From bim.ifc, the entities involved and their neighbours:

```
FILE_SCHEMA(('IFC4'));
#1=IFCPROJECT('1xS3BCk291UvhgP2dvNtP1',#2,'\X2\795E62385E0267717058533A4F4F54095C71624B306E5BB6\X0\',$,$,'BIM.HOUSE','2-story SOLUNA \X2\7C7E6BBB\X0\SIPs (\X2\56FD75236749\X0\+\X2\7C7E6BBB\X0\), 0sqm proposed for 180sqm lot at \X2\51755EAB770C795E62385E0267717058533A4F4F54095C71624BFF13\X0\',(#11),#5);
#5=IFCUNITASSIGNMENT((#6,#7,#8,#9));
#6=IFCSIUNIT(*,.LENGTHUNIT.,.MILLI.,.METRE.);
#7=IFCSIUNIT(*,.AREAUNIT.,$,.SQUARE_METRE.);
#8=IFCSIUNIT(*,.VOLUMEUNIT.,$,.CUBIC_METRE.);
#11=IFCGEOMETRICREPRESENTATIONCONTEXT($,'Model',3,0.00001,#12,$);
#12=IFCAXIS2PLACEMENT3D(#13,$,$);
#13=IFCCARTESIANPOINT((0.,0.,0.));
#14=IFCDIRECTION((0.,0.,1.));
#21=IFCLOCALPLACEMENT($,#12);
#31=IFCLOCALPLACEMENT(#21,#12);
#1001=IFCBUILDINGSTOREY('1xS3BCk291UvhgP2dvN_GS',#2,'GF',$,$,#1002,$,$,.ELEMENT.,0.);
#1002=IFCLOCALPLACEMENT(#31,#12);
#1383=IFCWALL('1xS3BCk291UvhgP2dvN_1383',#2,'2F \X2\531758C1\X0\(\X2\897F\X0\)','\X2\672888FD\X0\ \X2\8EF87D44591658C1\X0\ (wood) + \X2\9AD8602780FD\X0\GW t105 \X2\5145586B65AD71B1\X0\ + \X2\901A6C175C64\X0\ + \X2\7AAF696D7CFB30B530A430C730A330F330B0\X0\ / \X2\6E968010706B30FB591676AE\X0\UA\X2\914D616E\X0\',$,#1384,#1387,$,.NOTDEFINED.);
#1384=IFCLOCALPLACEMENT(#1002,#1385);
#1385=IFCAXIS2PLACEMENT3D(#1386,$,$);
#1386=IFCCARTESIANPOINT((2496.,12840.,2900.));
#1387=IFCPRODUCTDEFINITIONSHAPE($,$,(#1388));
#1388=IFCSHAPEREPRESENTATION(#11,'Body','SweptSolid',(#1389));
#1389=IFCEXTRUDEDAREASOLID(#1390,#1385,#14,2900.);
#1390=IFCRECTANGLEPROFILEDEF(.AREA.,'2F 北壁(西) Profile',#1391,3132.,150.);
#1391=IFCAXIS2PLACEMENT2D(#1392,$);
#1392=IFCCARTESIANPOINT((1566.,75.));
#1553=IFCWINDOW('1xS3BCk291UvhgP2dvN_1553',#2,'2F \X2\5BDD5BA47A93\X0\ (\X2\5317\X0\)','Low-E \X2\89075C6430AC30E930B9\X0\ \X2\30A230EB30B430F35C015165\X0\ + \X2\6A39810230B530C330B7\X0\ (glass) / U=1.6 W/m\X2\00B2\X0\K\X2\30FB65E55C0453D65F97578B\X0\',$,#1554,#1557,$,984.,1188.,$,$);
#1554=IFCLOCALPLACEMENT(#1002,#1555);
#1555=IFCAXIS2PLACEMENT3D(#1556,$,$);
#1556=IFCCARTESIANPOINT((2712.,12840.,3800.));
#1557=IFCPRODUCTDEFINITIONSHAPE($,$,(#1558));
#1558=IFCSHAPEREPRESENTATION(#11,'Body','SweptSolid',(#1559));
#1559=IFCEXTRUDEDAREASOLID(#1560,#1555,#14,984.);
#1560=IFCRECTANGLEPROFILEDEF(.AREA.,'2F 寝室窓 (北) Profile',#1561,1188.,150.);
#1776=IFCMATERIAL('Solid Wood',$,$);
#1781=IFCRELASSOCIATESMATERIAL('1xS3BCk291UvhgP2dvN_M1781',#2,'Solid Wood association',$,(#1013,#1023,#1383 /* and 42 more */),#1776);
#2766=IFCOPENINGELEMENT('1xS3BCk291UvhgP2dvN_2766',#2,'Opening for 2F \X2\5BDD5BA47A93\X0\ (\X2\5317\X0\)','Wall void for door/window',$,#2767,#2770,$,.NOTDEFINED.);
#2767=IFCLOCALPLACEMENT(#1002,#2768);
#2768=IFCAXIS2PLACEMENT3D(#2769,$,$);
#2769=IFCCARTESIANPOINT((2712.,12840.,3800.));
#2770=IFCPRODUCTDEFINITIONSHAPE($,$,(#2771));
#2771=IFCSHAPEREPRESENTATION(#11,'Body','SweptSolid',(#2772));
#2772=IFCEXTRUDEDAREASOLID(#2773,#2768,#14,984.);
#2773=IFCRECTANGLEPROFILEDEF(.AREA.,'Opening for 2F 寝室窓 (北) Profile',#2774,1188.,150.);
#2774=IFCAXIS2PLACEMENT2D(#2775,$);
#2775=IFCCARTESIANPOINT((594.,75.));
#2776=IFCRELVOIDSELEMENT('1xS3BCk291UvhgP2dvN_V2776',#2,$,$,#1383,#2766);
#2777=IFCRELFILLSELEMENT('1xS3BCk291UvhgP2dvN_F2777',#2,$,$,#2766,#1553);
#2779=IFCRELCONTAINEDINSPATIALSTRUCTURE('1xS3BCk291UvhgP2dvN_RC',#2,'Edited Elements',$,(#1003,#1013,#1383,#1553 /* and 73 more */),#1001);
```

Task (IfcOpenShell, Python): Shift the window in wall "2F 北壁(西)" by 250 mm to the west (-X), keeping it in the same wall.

```python
import ifcopenshell
import ifcopenshell.api.geometry
import ifcopenshell.util.placement
import ifcopenshell.util.unit

model = ifcopenshell.open("bim.ifc")
unit_scale = ifcopenshell.util.unit.calculate_unit_scale(model)

window = model.by_guid("1xS3BCk291UvhgP2dvN_1553")
opening = window.FillsVoids[0].RelatingOpeningElement
wall = opening.VoidsElements[0].RelatingBuildingElement

wall_matrix = ifcopenshell.util.placement.get_local_placement(wall.ObjectPlacement)
shift = wall_matrix[:3, 0] * -0.25 / unit_scale
before = ifcopenshell.util.placement.get_local_placement(window.ObjectPlacement)[:3, 3].copy()

# The window is not placed relative to its opening, so move both.
for product in (opening, window):
    matrix = ifcopenshell.util.placement.get_local_placement(product.ObjectPlacement)
    matrix[:3, 3] += shift
    ifcopenshell.api.geometry.edit_object_placement(model, product=product, matrix=matrix, is_si=False)

after = ifcopenshell.util.placement.get_local_placement(window.ObjectPlacement)[:3, 3]
print("window moved by", (after - before).round(3) + 0.0)

model.write("bim-out.ifc")
```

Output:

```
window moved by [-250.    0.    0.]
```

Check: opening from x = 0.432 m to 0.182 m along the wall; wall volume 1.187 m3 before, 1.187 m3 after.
